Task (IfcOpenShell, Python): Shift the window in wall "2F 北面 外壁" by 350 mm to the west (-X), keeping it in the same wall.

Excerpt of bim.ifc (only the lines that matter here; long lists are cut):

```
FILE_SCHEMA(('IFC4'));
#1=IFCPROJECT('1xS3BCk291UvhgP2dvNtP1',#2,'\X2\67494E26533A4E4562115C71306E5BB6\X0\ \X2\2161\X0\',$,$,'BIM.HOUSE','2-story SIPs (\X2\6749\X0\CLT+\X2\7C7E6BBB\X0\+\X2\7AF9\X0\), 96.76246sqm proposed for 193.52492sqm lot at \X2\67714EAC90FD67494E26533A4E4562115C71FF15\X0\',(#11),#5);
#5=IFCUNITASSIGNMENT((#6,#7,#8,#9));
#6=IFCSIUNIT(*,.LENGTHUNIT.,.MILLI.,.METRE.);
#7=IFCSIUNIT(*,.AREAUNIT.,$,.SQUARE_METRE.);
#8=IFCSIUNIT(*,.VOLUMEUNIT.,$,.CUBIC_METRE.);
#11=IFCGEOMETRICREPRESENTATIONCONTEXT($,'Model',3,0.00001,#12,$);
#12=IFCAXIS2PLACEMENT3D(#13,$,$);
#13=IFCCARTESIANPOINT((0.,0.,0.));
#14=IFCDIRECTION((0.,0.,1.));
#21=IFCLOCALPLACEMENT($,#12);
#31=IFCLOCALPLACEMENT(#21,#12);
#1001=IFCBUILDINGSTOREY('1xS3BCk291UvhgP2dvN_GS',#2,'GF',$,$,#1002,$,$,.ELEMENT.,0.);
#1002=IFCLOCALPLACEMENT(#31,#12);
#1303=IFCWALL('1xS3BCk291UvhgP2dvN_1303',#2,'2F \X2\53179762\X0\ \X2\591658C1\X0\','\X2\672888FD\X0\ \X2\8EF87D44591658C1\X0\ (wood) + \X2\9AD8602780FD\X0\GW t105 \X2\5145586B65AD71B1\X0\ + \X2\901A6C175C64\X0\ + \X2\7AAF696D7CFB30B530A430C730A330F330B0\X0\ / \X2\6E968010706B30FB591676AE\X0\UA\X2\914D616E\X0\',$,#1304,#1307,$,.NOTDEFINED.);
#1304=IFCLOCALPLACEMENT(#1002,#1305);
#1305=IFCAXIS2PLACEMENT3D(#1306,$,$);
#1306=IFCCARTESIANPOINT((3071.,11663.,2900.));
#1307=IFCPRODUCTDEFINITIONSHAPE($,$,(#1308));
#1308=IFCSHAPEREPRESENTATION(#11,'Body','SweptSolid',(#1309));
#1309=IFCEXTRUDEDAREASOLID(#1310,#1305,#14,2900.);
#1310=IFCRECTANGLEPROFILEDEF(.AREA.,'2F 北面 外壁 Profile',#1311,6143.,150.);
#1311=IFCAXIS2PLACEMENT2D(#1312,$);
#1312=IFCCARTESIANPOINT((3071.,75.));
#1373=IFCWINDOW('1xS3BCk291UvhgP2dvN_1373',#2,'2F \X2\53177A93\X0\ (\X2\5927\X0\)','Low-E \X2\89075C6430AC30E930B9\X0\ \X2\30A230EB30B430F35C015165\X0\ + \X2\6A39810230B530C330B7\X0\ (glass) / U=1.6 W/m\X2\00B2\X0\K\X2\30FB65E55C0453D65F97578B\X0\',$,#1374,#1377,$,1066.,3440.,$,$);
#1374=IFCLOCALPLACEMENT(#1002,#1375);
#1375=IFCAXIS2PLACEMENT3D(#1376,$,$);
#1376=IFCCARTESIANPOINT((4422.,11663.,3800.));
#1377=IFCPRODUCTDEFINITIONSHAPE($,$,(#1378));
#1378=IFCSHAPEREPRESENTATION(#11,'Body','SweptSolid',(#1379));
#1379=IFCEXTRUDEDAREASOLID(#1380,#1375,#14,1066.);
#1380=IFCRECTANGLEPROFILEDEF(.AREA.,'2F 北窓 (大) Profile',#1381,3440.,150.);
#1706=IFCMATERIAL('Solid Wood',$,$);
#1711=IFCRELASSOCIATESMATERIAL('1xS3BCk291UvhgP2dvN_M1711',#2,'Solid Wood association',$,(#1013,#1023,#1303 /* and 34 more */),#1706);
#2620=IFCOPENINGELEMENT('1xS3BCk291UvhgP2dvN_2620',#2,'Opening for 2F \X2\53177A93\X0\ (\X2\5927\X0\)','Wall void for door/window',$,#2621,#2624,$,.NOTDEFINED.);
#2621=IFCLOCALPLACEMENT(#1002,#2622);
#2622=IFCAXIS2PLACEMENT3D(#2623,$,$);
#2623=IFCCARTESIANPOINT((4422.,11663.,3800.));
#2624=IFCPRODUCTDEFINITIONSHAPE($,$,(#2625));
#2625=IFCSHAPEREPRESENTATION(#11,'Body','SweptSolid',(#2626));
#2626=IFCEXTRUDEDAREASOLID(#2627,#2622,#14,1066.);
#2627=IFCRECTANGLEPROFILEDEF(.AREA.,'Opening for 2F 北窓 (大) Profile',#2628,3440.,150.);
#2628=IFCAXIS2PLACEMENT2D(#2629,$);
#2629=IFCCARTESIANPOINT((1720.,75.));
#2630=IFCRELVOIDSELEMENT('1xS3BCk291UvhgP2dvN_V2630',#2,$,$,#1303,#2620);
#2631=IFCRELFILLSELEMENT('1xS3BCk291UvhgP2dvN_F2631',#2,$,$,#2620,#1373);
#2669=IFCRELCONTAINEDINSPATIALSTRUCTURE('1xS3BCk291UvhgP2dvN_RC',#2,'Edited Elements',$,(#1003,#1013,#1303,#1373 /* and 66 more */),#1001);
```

```python
import ifcopenshell
import ifcopenshell.api.geometry
import ifcopenshell.util.placement

model = ifcopenshell.open("bim.ifc")

window = model.by_guid("1xS3BCk291UvhgP2dvN_1373")
opening = window.FillsVoids[0].RelatingOpeningElement
wall = opening.VoidsElements[0].RelatingBuildingElement

wall_matrix = ifcopenshell.util.placement.get_local_placement(wall.ObjectPlacement)
shift = wall_matrix[:3, 0] * -350.0
before = ifcopenshell.util.placement.get_local_placement(window.ObjectPlacement)[:3, 3].copy()

# The window is not placed relative to its opening, so move both.
for product in (opening, window):
    matrix = ifcopenshell.util.placement.get_local_placement(product.ObjectPlacement)
    matrix[:3, 3] += shift
    ifcopenshell.api.geometry.edit_object_placement(model, product=product, matrix=matrix, is_si=False)

after = ifcopenshell.util.placement.get_local_placement(window.ObjectPlacement)[:3, 3]
print("window moved by", (after - before).round(3) + 0.0)

model.write("bim_rev.ifc")
```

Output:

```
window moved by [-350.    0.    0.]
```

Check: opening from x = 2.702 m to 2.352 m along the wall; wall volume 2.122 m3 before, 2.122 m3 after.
